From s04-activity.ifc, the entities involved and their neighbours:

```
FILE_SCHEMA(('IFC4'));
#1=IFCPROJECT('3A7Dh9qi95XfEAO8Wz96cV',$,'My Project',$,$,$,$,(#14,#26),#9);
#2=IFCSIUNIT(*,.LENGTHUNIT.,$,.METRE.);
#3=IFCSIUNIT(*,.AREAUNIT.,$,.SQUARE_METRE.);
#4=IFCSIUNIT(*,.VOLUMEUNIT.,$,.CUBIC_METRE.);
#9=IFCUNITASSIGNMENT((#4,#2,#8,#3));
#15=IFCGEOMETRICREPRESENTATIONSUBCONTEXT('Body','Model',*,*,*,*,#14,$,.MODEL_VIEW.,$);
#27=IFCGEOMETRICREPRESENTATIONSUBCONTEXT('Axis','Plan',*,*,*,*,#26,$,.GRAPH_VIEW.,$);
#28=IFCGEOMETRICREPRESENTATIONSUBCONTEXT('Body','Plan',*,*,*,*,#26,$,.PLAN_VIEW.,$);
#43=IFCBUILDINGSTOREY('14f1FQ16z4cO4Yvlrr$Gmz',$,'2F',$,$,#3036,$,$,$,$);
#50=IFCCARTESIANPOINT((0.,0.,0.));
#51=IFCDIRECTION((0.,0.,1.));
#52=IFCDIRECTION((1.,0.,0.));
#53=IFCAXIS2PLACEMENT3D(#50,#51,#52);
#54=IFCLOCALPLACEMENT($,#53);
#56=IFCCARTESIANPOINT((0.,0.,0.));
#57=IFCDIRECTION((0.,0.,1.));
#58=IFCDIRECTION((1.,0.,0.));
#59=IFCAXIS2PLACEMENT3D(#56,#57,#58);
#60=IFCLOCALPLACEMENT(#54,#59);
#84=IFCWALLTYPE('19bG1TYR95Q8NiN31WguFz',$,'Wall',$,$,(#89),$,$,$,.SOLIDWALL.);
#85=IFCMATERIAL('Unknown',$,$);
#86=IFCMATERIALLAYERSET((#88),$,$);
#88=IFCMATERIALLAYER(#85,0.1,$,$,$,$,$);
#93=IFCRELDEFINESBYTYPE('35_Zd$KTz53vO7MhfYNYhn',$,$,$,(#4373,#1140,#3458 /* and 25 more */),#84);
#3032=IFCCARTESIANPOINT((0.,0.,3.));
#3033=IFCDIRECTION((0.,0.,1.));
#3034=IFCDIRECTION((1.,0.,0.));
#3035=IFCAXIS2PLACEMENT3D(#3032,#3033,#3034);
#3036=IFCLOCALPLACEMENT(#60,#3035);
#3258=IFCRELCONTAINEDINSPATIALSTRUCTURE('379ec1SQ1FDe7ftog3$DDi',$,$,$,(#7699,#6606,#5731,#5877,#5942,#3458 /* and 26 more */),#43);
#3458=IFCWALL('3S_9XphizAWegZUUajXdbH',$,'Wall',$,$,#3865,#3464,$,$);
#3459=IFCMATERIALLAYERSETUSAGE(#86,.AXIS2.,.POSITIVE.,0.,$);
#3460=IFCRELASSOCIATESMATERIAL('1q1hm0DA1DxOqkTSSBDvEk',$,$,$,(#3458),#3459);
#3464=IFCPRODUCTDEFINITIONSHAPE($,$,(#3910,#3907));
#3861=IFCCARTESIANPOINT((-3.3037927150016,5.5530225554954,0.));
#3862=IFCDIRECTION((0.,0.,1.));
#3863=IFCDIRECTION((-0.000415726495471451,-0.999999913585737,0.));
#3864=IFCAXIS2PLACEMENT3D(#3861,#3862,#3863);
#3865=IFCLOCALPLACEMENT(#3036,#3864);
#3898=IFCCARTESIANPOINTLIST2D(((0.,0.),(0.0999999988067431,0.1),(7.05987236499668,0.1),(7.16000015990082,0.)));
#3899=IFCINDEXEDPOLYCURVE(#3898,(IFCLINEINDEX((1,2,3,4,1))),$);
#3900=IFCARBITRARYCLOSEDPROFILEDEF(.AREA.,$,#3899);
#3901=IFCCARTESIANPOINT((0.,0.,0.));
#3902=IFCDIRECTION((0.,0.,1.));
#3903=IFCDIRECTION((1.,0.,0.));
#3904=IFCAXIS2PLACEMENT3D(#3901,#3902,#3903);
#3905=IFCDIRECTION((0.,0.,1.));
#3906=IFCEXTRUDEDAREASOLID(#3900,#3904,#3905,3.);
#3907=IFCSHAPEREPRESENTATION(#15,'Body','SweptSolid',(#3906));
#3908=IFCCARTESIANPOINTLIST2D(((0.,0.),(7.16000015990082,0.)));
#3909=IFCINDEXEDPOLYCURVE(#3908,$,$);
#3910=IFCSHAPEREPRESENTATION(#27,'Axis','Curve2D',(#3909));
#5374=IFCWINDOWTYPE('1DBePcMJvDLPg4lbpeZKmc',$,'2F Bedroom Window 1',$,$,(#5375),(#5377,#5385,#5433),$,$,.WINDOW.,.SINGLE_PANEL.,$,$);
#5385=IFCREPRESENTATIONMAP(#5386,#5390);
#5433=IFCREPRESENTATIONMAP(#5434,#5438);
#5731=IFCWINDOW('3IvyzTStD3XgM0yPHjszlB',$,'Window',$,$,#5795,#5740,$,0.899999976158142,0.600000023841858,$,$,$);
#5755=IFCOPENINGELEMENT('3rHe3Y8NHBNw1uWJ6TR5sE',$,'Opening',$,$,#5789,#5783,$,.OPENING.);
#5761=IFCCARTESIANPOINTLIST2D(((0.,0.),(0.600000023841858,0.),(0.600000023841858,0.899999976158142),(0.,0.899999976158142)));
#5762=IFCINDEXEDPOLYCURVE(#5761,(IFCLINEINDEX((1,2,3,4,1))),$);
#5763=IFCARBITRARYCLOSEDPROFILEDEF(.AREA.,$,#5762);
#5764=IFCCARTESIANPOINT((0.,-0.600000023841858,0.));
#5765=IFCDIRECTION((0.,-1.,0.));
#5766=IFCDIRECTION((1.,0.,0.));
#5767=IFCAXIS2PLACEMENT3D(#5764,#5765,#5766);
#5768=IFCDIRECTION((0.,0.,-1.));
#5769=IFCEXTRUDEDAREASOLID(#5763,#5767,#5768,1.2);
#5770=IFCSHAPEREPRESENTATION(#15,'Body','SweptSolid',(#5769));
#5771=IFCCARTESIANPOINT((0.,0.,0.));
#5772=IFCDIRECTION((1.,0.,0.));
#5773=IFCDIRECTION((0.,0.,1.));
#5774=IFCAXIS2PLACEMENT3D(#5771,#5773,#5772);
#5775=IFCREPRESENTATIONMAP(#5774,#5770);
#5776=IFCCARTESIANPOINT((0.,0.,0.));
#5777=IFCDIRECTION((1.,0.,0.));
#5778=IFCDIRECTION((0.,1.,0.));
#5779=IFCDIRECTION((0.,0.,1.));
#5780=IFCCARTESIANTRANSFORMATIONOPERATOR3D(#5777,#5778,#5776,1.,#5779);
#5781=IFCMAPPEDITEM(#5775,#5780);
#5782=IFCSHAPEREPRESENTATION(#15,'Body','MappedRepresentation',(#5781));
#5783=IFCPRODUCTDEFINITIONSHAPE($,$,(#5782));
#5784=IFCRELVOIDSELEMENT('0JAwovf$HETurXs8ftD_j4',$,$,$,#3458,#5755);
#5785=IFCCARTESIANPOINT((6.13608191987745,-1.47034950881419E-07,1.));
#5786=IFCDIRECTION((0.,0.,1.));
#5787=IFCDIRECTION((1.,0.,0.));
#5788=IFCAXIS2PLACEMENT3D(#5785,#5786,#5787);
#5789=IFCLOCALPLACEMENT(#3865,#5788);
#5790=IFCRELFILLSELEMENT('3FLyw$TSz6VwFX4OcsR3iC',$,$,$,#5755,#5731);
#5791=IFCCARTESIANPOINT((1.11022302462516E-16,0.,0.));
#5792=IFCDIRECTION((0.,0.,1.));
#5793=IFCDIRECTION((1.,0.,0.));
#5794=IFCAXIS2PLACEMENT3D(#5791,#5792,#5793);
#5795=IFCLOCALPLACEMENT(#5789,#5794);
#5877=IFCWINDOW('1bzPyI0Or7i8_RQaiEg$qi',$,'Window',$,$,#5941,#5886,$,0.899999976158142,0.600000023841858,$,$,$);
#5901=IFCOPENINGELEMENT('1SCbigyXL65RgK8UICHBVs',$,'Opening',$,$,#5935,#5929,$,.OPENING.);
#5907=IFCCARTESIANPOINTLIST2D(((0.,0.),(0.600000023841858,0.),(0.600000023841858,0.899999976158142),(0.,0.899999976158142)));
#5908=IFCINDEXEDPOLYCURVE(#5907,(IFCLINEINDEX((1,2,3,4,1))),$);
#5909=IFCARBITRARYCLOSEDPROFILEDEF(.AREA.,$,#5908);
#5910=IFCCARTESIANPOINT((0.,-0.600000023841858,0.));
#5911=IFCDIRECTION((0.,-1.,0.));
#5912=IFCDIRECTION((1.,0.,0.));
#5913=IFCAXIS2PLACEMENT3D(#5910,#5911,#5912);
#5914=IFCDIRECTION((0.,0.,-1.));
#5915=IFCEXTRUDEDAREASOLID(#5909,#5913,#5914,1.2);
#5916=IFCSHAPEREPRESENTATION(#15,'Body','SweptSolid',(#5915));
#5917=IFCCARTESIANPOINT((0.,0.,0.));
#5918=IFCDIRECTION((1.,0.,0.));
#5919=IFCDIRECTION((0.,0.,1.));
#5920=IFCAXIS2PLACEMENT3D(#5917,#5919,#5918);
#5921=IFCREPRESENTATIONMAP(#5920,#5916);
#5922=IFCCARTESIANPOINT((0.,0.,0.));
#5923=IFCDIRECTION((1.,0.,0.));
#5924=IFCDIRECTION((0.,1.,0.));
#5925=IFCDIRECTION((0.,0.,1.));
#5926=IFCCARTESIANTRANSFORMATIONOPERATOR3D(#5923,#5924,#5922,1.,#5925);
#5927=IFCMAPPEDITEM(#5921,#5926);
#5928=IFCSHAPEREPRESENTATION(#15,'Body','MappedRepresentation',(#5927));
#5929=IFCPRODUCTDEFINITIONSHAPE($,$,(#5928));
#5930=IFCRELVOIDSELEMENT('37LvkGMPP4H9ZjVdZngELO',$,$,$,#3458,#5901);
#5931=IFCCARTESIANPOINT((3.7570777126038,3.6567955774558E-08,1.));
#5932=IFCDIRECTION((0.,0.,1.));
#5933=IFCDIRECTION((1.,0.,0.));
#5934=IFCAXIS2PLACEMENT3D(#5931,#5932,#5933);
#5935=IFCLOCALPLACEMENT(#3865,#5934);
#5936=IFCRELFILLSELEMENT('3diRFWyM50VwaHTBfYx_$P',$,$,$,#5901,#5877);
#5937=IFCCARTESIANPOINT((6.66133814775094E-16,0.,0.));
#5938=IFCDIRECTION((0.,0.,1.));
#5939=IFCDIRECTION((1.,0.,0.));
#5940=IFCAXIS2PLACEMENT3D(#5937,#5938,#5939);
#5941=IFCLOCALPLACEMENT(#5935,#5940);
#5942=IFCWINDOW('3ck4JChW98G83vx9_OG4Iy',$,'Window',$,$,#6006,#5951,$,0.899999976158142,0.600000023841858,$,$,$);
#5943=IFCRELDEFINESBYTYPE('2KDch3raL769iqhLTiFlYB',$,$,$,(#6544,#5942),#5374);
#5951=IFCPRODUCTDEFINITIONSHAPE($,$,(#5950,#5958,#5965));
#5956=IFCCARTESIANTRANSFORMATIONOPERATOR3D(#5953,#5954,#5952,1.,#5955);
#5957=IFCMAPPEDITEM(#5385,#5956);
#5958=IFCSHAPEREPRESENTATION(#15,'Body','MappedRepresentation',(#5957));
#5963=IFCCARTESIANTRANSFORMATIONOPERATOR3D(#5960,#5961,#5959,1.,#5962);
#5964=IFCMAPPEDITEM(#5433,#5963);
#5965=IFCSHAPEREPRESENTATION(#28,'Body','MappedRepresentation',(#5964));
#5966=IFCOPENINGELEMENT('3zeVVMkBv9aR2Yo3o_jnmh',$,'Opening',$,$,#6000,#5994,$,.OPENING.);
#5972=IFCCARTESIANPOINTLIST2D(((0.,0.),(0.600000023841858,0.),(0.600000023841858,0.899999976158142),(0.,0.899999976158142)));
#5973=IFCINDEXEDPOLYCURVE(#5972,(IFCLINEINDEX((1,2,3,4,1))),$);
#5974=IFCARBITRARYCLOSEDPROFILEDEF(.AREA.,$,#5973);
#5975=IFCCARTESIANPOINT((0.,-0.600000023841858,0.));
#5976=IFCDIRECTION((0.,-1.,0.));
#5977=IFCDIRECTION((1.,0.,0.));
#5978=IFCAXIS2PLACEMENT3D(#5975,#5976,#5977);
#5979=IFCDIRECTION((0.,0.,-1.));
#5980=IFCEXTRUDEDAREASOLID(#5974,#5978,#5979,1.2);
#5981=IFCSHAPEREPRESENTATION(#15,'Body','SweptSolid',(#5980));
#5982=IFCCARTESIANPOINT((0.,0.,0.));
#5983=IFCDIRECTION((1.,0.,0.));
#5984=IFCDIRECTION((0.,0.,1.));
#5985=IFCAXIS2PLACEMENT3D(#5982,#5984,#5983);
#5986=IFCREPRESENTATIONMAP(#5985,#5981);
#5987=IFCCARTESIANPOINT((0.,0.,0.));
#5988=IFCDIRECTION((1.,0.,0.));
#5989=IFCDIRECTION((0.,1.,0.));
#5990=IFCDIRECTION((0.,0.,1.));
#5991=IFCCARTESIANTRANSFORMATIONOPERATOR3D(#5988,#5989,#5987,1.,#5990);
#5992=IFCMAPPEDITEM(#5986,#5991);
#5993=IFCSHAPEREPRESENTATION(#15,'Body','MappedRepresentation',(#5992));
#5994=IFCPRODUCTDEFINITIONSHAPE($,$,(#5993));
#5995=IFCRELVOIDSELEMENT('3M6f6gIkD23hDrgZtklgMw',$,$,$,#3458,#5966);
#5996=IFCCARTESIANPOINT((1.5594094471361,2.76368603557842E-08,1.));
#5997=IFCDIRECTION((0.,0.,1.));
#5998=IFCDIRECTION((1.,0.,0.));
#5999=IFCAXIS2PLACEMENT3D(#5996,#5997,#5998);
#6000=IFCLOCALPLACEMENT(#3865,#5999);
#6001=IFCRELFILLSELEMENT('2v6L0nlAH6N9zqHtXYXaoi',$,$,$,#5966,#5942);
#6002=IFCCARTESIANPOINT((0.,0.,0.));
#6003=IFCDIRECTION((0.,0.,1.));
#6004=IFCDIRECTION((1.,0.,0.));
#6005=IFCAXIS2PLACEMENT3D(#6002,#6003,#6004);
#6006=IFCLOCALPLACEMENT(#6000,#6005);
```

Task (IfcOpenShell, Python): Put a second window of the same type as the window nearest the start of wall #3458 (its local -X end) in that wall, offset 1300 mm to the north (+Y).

```python
import ifcopenshell
import ifcopenshell.api.feature
import ifcopenshell.api.geometry
import ifcopenshell.api.root
import ifcopenshell.geom
import ifcopenshell.util.element
import ifcopenshell.util.placement
import ifcopenshell.util.shape

model = ifcopenshell.open("s04-activity.ifc")
settings = ifcopenshell.geom.settings()


def volume(element):
    """Net volume in cubic metres, openings subtracted."""
    shape = ifcopenshell.geom.create_shape(settings, element)
    return ifcopenshell.util.shape.get_volume(shape.geometry)


window = model.by_guid("3ck4JChW98G83vx9_OG4Iy")
opening = window.FillsVoids[0].RelatingOpeningElement
wall = opening.VoidsElements[0].RelatingBuildingElement
before = volume(wall)
shift = ifcopenshell.util.placement.get_local_placement(wall.ObjectPlacement)[:3, 0] * -1.3

# copy_class copies the void relationship, type, container and properties, but no geometry.
new_opening = ifcopenshell.api.root.copy_class(model, product=opening)
new_opening.Representation = ifcopenshell.util.element.copy_deep(
    model, opening.Representation, exclude=["IfcGeometricRepresentationContext", "IfcRepresentationMap"]
)
new_window = ifcopenshell.api.root.copy_class(model, product=window)
new_window.Representation = ifcopenshell.util.element.copy_deep(
    model, window.Representation, exclude=["IfcGeometricRepresentationContext", "IfcRepresentationMap"]
)
ifcopenshell.api.feature.add_filling(model, opening=new_opening, element=new_window)

for old, new in ((opening, new_opening), (window, new_window)):
    matrix = ifcopenshell.util.placement.get_local_placement(old.ObjectPlacement)
    matrix[:3, 3] += shift
    ifcopenshell.api.geometry.edit_object_placement(model, product=new, matrix=matrix, is_si=False)

after = volume(wall)

print(f"wall volume {before:.3f} -> {after:.3f} m3")

model.write("s04-activity_updated.ifc")
```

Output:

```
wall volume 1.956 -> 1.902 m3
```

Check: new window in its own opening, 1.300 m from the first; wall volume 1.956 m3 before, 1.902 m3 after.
